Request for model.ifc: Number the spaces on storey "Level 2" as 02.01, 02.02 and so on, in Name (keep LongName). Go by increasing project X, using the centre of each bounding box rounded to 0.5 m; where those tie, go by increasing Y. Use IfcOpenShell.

First a look at what the model holds.

```python
import ifcopenshell
import ifcopenshell.util.element
import ifcopenshell.util.placement

model = ifcopenshell.open("model.ifc")
print(model.schema)
storey = next(s for s in model.by_type("IfcBuildingStorey") if s.Name == "Level 2")
spaces = [e for e in ifcopenshell.util.element.get_decomposition(storey) if e.is_a("IfcSpace")]
for e in sorted(spaces, key=lambda e: e.id()):
    origin = ifcopenshell.util.placement.get_local_placement(e.ObjectPlacement)[:3, 3]
    print(e.id(), e.Name, e.LongName, origin.round(2) + 0.0, sep=" | ")
```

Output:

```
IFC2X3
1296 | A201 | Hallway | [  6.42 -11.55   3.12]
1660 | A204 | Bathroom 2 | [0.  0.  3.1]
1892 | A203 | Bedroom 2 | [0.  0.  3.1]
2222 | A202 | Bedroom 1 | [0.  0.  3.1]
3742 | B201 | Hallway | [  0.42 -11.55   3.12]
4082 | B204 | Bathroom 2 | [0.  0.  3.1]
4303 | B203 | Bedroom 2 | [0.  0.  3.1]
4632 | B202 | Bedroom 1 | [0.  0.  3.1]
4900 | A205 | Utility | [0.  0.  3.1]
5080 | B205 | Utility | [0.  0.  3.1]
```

```python
import ifcopenshell
import ifcopenshell.geom
import ifcopenshell.util.element
import ifcopenshell.util.shape

model = ifcopenshell.open("model.ifc")
settings = ifcopenshell.geom.settings()
settings.set("use-world-coords", True)


def centre(element):
    shape = ifcopenshell.geom.create_shape(settings, element)
    return ifcopenshell.util.shape.get_bbox_centroid(shape.geometry)


storey = next(s for s in model.by_type("IfcBuildingStorey") if s.Name == "Level 2")
spaces = [e for e in ifcopenshell.util.element.get_decomposition(storey) if e.is_a("IfcSpace")]

# Insertion points can sit at a corner or the storey origin, so sort by the geometry (in metres).
centres = {e: centre(e) for e in spaces}
spaces.sort(key=lambda e: (round(centres[e][0] / 0.5), centres[e][1]))

for i, e in enumerate(spaces, start=1):
    number = f"02.{i:02d}"
    e.Name = number
    print(e.id(), number)

model.write("model_rev.ifc")
```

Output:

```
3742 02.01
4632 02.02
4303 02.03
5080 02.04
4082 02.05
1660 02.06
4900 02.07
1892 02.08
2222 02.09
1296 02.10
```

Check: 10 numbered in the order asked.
